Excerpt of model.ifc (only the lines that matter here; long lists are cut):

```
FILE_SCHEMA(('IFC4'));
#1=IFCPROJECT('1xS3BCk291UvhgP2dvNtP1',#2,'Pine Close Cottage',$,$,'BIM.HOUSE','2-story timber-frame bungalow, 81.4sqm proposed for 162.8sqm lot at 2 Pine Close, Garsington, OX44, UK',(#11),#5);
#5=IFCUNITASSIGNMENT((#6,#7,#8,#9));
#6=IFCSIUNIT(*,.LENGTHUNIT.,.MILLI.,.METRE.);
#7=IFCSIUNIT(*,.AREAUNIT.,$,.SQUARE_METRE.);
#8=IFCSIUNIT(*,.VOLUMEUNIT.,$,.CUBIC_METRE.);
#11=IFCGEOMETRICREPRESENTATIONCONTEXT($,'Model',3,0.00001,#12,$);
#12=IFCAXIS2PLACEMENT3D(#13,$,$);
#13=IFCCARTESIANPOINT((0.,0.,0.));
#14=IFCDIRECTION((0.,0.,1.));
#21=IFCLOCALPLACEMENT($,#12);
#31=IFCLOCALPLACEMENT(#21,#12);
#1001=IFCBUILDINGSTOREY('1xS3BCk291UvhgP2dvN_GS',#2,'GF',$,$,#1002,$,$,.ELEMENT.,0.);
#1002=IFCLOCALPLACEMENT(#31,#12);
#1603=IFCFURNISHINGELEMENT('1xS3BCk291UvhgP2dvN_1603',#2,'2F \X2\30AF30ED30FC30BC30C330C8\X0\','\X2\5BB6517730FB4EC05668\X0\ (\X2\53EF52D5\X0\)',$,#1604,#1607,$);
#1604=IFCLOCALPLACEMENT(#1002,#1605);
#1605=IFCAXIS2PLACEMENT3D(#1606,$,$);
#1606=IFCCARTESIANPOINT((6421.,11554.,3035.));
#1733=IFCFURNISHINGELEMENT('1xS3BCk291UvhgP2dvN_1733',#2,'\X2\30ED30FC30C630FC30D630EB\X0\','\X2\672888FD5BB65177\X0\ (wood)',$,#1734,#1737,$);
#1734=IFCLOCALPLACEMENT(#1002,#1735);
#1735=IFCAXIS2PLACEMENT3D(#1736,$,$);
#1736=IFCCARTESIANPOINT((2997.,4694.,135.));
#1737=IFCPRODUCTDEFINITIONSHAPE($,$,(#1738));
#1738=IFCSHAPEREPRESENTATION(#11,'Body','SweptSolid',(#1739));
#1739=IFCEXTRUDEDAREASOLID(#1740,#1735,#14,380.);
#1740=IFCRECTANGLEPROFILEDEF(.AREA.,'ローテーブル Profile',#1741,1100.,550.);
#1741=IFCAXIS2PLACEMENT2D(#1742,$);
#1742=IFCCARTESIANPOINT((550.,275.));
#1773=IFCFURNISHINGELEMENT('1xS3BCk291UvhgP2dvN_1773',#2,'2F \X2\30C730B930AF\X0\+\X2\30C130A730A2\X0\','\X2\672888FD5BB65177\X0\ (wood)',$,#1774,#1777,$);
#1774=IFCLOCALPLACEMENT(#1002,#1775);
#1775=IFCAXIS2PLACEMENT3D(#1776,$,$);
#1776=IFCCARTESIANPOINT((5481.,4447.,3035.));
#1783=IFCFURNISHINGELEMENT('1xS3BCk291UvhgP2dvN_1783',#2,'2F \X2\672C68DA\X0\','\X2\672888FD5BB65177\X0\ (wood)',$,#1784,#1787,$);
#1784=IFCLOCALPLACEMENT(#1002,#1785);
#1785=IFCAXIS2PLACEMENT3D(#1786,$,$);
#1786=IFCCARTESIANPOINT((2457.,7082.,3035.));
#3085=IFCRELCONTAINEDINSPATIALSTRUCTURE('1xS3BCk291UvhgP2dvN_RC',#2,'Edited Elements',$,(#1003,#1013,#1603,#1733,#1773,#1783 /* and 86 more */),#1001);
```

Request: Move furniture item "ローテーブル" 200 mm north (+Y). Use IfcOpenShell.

```python
import ifcopenshell
import ifcopenshell.api.geometry
import ifcopenshell.util.placement

model = ifcopenshell.open("model.ifc")

item = model.by_guid("1xS3BCk291UvhgP2dvN_1733")
matrix = ifcopenshell.util.placement.get_local_placement(item.ObjectPlacement)
matrix[1, 3] += 200.0
ifcopenshell.api.geometry.edit_object_placement(model, product=item, matrix=matrix, is_si=False)

print(ifcopenshell.util.placement.get_local_placement(item.ObjectPlacement).round(3) + 0.0)

model.write("model_v2.ifc")
```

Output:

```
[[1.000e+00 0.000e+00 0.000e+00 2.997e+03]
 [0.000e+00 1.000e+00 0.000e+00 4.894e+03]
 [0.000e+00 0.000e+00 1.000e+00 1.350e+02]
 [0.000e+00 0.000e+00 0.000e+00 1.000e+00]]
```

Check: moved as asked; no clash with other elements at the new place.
